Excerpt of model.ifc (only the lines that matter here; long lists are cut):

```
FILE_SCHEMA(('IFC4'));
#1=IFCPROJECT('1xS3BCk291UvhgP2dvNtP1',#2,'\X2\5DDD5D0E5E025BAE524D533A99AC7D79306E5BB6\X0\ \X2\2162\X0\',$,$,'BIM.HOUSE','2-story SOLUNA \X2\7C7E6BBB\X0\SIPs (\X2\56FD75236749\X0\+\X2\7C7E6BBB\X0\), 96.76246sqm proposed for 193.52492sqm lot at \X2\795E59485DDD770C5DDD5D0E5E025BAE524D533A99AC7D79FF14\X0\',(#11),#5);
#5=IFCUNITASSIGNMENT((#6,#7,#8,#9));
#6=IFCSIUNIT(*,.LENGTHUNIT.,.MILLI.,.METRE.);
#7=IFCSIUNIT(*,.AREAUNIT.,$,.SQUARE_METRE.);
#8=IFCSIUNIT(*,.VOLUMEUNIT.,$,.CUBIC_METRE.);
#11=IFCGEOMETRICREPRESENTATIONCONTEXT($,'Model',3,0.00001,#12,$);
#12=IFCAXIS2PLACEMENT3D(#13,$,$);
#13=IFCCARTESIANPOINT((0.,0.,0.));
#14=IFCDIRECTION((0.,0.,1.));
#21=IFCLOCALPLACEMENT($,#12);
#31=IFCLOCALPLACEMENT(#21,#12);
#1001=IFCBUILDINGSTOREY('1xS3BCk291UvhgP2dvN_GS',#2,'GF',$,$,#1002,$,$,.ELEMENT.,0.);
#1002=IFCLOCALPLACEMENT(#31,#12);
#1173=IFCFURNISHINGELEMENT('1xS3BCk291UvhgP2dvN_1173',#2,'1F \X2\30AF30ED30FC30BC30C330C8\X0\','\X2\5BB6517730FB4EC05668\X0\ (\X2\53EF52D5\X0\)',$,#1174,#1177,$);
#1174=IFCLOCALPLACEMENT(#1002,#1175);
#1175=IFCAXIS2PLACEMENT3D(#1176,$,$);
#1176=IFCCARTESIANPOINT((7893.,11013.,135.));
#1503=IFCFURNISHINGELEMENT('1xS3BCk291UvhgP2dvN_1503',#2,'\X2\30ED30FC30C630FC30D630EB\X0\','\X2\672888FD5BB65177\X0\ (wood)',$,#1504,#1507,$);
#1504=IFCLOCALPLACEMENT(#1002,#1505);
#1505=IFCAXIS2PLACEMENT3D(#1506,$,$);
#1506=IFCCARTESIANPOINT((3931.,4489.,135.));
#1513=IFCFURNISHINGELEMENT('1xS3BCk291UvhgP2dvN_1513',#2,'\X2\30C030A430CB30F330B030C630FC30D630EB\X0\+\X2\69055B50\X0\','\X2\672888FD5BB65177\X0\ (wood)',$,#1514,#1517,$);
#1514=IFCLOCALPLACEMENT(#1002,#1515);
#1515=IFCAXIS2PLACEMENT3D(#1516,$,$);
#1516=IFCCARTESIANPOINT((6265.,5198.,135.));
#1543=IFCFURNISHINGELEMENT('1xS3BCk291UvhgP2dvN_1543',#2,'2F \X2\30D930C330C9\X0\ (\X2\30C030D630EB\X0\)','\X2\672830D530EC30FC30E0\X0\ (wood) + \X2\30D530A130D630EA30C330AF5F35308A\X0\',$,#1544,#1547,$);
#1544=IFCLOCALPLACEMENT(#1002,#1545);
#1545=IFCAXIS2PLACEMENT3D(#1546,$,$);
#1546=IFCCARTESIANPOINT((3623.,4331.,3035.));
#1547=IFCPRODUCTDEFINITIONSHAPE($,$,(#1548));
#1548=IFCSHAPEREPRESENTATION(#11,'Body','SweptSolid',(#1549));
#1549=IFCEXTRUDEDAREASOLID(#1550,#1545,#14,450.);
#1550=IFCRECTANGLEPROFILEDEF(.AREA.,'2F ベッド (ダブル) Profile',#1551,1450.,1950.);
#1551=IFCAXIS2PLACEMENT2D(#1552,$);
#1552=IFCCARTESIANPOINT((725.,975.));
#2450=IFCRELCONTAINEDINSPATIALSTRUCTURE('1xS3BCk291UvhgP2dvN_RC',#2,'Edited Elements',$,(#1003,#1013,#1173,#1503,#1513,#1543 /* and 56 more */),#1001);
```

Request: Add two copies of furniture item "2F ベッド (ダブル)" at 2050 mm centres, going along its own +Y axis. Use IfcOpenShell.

```python
import ifcopenshell
import ifcopenshell.api.geometry
import ifcopenshell.api.root
import ifcopenshell.util.element
import ifcopenshell.util.placement
import ifcopenshell.util.unit

model = ifcopenshell.open("model.ifc")
unit_scale = ifcopenshell.util.unit.calculate_unit_scale(model)


def reuse_history(source, copy):
    """copy_class also copies each property set's owner history, people and application; keep the originals."""
    for rel in copy.IsDefinedBy:
        if rel.is_a("IfcRelDefinesByProperties") and (history := rel.RelatingPropertyDefinition.OwnerHistory):
            rel.RelatingPropertyDefinition.OwnerHistory = source.OwnerHistory
            ifcopenshell.util.element.remove_deep2(model, history)


source = model.by_guid("1xS3BCk291UvhgP2dvN_1543")
base = ifcopenshell.util.placement.get_local_placement(source.ObjectPlacement)
step = base[:3, 1] * 2.05 / unit_scale

for i in range(1, 3):
    copy = ifcopenshell.api.root.copy_class(model, product=source)
    copy.Representation = ifcopenshell.util.element.copy_deep(
        model, source.Representation, exclude=["IfcGeometricRepresentationContext", "IfcRepresentationMap"]
    )
    reuse_history(source, copy)
    matrix = base.copy()
    matrix[:3, 3] += i * step
    print("added at", matrix[:3, 3].round(3) + 0.0)
    ifcopenshell.api.geometry.edit_object_placement(model, product=copy, matrix=matrix, is_si=False)

model.write("model_rev.ifc")
```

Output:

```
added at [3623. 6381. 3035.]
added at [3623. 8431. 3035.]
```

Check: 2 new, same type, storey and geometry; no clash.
